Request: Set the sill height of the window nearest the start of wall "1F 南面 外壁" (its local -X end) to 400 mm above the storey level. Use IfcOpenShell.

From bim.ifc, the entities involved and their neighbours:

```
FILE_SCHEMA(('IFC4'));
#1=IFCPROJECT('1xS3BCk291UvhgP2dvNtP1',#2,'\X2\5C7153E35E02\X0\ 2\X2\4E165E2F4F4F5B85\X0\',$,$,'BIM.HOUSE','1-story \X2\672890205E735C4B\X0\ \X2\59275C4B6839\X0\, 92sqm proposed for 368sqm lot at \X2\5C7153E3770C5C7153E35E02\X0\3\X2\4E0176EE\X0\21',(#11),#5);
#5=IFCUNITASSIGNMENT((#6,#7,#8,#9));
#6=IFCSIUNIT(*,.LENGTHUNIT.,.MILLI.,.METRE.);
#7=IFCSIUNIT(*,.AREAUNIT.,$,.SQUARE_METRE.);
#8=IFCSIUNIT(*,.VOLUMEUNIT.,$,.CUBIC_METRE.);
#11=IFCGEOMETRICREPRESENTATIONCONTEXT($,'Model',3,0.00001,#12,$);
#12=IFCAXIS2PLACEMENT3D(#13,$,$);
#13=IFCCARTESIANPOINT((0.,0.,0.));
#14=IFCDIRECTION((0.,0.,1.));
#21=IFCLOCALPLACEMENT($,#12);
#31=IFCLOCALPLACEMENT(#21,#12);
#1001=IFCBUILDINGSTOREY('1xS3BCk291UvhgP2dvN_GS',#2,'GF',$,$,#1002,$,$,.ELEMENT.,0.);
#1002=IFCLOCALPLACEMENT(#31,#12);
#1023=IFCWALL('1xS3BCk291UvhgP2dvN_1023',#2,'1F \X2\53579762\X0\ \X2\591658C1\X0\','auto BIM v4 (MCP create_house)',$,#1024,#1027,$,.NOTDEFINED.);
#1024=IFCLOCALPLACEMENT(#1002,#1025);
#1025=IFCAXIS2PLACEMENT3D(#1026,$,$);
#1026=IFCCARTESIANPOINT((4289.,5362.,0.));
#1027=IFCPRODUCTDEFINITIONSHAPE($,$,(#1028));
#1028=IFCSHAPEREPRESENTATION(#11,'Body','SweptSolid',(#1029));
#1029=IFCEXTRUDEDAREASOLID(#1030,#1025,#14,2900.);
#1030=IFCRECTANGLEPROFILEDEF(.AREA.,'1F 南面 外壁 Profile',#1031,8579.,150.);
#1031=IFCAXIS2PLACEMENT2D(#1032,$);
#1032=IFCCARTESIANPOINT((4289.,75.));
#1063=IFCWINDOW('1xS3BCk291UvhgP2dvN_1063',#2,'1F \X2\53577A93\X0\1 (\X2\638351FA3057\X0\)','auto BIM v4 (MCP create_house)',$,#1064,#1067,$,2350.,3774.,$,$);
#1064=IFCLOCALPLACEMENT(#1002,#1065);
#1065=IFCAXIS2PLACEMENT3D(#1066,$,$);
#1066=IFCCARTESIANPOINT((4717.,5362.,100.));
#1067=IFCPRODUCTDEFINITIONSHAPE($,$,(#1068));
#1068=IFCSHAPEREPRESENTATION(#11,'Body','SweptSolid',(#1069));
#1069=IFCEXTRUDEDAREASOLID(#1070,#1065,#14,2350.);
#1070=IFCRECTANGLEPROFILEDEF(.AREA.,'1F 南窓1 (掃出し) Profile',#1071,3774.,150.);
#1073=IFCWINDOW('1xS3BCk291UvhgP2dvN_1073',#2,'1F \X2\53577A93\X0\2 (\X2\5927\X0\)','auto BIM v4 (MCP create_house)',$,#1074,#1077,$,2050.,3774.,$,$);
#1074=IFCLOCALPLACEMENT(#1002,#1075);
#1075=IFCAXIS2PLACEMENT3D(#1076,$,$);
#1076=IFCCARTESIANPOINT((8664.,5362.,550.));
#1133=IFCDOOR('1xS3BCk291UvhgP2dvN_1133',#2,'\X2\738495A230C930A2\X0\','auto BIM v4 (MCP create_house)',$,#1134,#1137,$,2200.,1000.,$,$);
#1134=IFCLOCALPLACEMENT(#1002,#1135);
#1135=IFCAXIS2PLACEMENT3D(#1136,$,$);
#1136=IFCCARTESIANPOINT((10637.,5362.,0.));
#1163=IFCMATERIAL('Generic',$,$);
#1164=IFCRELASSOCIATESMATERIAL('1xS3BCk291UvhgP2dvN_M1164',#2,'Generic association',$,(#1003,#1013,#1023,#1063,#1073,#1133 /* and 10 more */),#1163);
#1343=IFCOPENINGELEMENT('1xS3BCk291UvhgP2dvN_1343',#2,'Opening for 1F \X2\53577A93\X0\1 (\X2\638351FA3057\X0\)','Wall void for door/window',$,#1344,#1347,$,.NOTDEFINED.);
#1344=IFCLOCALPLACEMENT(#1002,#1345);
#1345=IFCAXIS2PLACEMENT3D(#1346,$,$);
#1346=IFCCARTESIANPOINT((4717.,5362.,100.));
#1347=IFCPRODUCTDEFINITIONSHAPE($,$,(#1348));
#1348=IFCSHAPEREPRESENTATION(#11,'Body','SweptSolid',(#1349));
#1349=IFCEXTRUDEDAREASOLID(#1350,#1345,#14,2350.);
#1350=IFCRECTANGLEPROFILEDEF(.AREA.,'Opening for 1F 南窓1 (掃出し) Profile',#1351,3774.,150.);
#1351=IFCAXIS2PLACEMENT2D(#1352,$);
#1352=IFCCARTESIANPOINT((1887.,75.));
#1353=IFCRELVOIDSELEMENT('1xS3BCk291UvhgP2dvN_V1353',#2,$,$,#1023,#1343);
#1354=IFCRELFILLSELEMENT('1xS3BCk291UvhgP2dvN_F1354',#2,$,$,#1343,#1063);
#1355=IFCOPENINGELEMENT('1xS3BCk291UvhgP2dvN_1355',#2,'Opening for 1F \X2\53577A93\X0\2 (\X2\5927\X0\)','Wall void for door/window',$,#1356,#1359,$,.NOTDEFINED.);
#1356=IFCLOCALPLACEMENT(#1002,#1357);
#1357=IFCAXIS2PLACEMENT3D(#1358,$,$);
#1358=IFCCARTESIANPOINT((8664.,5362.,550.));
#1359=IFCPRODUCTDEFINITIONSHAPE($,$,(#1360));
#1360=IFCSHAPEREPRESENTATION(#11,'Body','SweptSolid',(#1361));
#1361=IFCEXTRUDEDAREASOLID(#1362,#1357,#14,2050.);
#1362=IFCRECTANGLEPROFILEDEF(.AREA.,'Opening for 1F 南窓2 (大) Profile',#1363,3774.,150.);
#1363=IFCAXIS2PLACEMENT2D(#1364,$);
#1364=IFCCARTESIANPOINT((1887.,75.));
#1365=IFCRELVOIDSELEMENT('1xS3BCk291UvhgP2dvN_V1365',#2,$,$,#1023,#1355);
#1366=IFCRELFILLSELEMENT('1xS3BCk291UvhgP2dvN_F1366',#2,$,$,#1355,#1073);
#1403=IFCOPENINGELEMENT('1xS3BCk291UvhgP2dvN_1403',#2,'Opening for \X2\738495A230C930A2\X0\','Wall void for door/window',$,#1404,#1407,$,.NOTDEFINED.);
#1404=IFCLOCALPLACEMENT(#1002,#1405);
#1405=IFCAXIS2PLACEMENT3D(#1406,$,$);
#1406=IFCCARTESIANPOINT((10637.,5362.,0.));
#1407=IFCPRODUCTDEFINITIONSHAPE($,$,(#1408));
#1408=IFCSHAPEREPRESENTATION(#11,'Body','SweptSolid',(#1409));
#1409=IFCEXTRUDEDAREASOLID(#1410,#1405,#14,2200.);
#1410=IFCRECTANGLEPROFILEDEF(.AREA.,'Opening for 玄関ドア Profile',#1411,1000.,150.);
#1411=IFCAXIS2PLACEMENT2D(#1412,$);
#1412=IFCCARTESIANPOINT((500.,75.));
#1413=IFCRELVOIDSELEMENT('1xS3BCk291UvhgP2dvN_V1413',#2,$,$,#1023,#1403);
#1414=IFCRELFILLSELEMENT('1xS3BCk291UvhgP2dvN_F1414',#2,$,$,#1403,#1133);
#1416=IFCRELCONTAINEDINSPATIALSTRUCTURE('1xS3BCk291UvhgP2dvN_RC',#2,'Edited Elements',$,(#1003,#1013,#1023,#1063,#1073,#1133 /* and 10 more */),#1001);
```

```python
import numpy as np
import ifcopenshell
import ifcopenshell.api.geometry
import ifcopenshell.geom
import ifcopenshell.util.element
import ifcopenshell.util.placement
import ifcopenshell.util.shape
import ifcopenshell.util.unit

model = ifcopenshell.open("bim.ifc")
unit_scale = ifcopenshell.util.unit.calculate_unit_scale(model)

window = model.by_id(1063)
opening = window.FillsVoids[0].RelatingOpeningElement
storey = ifcopenshell.util.element.get_container(window, ifc_class="IfcBuildingStorey")
level = ifcopenshell.util.placement.get_local_placement(storey.ObjectPlacement)[2, 3]

# The opening's origin need not be at the sill, so measure its lowest point.
shape = ifcopenshell.geom.create_shape(ifcopenshell.geom.settings(), opening)
bottom = ifcopenshell.util.shape.get_shape_bottom_elevation(shape, shape.geometry) / unit_scale
dz = level + 400.0 - bottom

shift = np.array([0.0, 0.0, dz])
# The window is not placed relative to its opening, so move both.
for product in (opening, window):
    matrix = ifcopenshell.util.placement.get_local_placement(product.ObjectPlacement)
    matrix[:3, 3] += shift
    ifcopenshell.api.geometry.edit_object_placement(model, product=product, matrix=matrix, is_si=False)

print(f"moved by {dz * unit_scale:+.3f} m")

model.write("bim_v2.ifc")
```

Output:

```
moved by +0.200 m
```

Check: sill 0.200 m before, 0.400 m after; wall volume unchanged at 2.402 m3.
